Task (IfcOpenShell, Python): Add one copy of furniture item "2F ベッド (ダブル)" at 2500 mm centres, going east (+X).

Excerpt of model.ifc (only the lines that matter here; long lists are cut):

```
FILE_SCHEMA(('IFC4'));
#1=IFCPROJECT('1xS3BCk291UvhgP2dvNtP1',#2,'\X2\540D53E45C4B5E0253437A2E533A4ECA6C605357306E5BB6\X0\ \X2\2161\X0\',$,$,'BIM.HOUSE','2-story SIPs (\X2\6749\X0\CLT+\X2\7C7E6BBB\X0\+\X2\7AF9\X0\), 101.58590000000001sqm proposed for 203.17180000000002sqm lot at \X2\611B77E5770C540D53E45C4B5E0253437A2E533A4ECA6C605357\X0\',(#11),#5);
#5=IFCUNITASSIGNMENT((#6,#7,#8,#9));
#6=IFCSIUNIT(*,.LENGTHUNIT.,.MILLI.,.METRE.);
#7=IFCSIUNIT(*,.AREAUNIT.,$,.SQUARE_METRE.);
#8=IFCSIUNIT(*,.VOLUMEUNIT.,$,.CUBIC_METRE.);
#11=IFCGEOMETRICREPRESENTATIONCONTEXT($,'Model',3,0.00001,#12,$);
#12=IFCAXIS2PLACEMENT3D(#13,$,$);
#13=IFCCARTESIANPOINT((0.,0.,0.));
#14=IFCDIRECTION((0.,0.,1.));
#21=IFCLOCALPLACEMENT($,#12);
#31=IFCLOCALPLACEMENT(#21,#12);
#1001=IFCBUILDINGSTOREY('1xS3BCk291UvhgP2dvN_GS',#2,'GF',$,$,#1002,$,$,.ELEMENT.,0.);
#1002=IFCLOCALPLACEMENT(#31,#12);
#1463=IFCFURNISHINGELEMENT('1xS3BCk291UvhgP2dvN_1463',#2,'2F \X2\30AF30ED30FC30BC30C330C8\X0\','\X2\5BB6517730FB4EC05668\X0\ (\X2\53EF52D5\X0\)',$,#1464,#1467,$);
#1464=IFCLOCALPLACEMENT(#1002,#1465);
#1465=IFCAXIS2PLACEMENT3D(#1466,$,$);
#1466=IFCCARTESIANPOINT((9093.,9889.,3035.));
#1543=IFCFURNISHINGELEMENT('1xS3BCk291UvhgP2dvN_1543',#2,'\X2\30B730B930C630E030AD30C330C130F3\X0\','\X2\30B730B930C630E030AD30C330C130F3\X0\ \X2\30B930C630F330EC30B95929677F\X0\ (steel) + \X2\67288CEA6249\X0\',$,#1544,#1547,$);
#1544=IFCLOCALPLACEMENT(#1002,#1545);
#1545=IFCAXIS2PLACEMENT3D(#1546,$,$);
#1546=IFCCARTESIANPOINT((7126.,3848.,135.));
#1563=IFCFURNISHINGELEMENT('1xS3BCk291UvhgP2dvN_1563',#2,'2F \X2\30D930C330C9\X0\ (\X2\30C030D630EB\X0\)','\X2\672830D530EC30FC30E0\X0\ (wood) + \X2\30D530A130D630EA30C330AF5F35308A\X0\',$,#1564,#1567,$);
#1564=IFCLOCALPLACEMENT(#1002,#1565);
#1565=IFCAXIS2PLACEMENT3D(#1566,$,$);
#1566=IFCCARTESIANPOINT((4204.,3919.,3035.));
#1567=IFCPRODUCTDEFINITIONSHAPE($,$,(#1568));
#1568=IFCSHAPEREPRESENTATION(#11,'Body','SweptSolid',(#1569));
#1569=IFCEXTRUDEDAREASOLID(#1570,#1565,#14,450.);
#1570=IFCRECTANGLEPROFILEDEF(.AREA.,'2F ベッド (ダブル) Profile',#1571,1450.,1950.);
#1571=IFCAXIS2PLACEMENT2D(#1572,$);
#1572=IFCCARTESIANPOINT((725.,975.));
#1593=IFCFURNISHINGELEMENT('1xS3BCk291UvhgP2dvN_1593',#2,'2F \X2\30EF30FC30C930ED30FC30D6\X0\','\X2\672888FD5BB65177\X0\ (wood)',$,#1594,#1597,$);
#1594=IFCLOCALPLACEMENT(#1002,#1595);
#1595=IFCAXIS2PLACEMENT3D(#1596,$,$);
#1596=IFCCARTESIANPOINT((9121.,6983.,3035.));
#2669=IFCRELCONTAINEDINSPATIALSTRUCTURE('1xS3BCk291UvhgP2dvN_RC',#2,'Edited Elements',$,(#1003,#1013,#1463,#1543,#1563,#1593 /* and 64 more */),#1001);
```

```python
import numpy as np
import ifcopenshell
import ifcopenshell.api.geometry
import ifcopenshell.api.root
import ifcopenshell.util.element
import ifcopenshell.util.placement
import ifcopenshell.util.unit

model = ifcopenshell.open("model.ifc")
unit_scale = ifcopenshell.util.unit.calculate_unit_scale(model)


def reuse_history(source, copy):
    """copy_class also copies each property set's owner history, people and application; keep the originals."""
    for rel in copy.IsDefinedBy:
        if rel.is_a("IfcRelDefinesByProperties") and (history := rel.RelatingPropertyDefinition.OwnerHistory):
            rel.RelatingPropertyDefinition.OwnerHistory = source.OwnerHistory
            ifcopenshell.util.element.remove_deep2(model, history)


source = model.by_id(1563)
base = ifcopenshell.util.placement.get_local_placement(source.ObjectPlacement)
step = np.array([1.0, 0.0, 0.0]) * 2.5 / unit_scale

for i in range(1, 2):
    copy = ifcopenshell.api.root.copy_class(model, product=source)
    copy.Representation = ifcopenshell.util.element.copy_deep(
        model, source.Representation, exclude=["IfcGeometricRepresentationContext", "IfcRepresentationMap"]
    )
    reuse_history(source, copy)
    matrix = base.copy()
    matrix[:3, 3] += i * step
    print("added at", matrix[:3, 3].round(3) + 0.0)
    ifcopenshell.api.geometry.edit_object_placement(model, product=copy, matrix=matrix, is_si=False)

model.write("model_updated.ifc")
```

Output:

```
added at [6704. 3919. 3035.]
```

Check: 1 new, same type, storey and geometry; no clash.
